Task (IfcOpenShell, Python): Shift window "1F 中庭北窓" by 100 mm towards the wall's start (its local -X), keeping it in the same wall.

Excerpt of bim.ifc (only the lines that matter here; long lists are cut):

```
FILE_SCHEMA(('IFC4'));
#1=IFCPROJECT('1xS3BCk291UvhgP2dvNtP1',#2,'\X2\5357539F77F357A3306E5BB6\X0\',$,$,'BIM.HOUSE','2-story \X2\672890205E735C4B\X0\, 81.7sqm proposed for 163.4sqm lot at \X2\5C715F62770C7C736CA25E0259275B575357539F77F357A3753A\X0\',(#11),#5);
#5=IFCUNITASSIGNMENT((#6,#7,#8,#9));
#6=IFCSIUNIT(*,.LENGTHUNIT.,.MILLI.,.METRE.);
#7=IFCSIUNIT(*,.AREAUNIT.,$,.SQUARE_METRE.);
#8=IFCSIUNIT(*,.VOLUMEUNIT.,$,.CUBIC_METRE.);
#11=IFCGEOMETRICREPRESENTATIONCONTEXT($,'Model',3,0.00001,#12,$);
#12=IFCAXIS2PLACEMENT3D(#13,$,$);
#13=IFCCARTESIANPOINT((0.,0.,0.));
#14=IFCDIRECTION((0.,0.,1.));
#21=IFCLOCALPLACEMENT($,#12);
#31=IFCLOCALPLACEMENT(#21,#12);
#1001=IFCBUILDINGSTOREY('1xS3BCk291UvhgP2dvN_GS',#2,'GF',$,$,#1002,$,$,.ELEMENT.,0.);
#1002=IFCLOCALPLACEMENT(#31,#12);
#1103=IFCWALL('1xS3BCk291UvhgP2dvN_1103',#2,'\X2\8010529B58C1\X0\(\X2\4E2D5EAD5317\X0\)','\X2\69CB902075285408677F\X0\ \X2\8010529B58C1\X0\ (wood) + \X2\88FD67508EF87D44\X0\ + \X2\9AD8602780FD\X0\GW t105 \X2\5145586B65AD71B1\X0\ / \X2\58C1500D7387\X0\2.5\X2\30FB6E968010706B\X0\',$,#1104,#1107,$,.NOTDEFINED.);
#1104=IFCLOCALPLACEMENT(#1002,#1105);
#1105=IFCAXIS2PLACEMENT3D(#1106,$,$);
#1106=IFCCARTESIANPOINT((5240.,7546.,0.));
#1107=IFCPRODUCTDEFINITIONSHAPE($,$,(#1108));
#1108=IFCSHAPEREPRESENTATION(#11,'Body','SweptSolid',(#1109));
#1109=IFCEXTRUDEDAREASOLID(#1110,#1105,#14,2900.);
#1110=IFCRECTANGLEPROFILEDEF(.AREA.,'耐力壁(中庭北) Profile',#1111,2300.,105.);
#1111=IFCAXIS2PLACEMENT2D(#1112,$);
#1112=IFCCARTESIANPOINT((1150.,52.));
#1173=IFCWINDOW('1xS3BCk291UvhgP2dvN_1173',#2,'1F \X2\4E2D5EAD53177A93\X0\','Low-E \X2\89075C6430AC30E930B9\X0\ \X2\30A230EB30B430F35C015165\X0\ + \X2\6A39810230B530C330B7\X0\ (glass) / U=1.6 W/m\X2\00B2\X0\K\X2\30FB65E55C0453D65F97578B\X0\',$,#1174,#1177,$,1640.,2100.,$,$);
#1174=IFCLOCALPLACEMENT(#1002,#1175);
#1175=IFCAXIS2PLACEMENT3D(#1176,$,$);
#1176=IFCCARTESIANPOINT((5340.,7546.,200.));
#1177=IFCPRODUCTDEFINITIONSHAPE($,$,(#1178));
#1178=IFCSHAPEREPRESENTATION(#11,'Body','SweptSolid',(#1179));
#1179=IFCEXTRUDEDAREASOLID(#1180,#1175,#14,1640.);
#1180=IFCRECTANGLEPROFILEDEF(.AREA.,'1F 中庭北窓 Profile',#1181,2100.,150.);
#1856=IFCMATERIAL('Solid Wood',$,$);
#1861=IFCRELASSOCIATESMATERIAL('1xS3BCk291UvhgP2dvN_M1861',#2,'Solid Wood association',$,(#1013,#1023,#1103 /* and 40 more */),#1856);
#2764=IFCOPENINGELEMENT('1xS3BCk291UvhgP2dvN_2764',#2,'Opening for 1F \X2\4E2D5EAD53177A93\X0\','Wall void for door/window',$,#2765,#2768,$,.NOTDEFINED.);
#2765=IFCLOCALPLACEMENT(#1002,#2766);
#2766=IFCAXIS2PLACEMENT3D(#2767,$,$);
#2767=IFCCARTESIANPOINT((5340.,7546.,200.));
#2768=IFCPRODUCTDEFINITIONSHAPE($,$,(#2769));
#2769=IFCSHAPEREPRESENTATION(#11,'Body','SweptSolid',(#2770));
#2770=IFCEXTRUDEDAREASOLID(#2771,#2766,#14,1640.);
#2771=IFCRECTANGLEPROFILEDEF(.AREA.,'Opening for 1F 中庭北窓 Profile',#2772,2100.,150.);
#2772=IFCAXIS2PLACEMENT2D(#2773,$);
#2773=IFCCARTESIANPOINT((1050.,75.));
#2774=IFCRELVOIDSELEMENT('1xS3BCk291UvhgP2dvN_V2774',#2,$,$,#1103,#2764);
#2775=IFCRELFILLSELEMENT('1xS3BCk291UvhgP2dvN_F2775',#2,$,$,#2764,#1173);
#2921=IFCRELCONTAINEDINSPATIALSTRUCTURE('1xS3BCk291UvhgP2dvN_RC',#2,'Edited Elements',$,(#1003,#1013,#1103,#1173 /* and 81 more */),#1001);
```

```python
import ifcopenshell
import ifcopenshell.api.geometry
import ifcopenshell.util.placement

model = ifcopenshell.open("bim.ifc")

window = model.by_id(1173)
opening = window.FillsVoids[0].RelatingOpeningElement
wall = opening.VoidsElements[0].RelatingBuildingElement

wall_matrix = ifcopenshell.util.placement.get_local_placement(wall.ObjectPlacement)
shift = wall_matrix[:3, 0] * -100.0
before = ifcopenshell.util.placement.get_local_placement(window.ObjectPlacement)[:3, 3].copy()

# The window is not placed relative to its opening, so move both.
for product in (opening, window):
    matrix = ifcopenshell.util.placement.get_local_placement(product.ObjectPlacement)
    matrix[:3, 3] += shift
    ifcopenshell.api.geometry.edit_object_placement(model, product=product, matrix=matrix, is_si=False)

after = ifcopenshell.util.placement.get_local_placement(window.ObjectPlacement)[:3, 3]
print("window moved by", (after - before).round(3) + 0.0)

model.write("bim-out.ifc")
```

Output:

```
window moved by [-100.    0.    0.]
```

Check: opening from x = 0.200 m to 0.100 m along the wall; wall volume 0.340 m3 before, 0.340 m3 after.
